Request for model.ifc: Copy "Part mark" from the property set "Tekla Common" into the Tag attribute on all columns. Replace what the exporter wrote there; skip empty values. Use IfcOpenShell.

First a look at what the model holds.

```python
import ifcopenshell
import ifcopenshell.util.element

model = ifcopenshell.open("model.ifc")
print(model.schema)
columns = model.by_type("IfcColumn")
print(len(columns), "columns")
for e in columns[:8]:
    source = ifcopenshell.util.element.get_pset(e, "Tekla Common", "Part mark")
    target = e.Tag
    print(e.id(), repr(source), repr(target), sep=" | ")
```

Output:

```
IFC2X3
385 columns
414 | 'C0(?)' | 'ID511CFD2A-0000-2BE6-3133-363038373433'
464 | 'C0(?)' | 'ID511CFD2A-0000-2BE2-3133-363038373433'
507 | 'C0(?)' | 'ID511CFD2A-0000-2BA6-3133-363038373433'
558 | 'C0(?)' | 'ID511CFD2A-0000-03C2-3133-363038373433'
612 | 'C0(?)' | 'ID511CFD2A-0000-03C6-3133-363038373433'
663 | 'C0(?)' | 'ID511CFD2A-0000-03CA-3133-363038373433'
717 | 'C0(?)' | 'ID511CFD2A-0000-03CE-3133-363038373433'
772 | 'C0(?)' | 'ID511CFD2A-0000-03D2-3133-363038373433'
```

```python
import ifcopenshell
import ifcopenshell.util.element

model = ifcopenshell.open("model.ifc")

count = 0
for e in model.by_type("IfcColumn"):
    value = ifcopenshell.util.element.get_pset(e, "Tekla Common", "Part mark")
    current = e.Tag
    if not value or not value.strip() or current == value:
        continue
    e.Tag = value
    count += 1

print(count, "columns updated")

model.write("model_rev.ifc")
```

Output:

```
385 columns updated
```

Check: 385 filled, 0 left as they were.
